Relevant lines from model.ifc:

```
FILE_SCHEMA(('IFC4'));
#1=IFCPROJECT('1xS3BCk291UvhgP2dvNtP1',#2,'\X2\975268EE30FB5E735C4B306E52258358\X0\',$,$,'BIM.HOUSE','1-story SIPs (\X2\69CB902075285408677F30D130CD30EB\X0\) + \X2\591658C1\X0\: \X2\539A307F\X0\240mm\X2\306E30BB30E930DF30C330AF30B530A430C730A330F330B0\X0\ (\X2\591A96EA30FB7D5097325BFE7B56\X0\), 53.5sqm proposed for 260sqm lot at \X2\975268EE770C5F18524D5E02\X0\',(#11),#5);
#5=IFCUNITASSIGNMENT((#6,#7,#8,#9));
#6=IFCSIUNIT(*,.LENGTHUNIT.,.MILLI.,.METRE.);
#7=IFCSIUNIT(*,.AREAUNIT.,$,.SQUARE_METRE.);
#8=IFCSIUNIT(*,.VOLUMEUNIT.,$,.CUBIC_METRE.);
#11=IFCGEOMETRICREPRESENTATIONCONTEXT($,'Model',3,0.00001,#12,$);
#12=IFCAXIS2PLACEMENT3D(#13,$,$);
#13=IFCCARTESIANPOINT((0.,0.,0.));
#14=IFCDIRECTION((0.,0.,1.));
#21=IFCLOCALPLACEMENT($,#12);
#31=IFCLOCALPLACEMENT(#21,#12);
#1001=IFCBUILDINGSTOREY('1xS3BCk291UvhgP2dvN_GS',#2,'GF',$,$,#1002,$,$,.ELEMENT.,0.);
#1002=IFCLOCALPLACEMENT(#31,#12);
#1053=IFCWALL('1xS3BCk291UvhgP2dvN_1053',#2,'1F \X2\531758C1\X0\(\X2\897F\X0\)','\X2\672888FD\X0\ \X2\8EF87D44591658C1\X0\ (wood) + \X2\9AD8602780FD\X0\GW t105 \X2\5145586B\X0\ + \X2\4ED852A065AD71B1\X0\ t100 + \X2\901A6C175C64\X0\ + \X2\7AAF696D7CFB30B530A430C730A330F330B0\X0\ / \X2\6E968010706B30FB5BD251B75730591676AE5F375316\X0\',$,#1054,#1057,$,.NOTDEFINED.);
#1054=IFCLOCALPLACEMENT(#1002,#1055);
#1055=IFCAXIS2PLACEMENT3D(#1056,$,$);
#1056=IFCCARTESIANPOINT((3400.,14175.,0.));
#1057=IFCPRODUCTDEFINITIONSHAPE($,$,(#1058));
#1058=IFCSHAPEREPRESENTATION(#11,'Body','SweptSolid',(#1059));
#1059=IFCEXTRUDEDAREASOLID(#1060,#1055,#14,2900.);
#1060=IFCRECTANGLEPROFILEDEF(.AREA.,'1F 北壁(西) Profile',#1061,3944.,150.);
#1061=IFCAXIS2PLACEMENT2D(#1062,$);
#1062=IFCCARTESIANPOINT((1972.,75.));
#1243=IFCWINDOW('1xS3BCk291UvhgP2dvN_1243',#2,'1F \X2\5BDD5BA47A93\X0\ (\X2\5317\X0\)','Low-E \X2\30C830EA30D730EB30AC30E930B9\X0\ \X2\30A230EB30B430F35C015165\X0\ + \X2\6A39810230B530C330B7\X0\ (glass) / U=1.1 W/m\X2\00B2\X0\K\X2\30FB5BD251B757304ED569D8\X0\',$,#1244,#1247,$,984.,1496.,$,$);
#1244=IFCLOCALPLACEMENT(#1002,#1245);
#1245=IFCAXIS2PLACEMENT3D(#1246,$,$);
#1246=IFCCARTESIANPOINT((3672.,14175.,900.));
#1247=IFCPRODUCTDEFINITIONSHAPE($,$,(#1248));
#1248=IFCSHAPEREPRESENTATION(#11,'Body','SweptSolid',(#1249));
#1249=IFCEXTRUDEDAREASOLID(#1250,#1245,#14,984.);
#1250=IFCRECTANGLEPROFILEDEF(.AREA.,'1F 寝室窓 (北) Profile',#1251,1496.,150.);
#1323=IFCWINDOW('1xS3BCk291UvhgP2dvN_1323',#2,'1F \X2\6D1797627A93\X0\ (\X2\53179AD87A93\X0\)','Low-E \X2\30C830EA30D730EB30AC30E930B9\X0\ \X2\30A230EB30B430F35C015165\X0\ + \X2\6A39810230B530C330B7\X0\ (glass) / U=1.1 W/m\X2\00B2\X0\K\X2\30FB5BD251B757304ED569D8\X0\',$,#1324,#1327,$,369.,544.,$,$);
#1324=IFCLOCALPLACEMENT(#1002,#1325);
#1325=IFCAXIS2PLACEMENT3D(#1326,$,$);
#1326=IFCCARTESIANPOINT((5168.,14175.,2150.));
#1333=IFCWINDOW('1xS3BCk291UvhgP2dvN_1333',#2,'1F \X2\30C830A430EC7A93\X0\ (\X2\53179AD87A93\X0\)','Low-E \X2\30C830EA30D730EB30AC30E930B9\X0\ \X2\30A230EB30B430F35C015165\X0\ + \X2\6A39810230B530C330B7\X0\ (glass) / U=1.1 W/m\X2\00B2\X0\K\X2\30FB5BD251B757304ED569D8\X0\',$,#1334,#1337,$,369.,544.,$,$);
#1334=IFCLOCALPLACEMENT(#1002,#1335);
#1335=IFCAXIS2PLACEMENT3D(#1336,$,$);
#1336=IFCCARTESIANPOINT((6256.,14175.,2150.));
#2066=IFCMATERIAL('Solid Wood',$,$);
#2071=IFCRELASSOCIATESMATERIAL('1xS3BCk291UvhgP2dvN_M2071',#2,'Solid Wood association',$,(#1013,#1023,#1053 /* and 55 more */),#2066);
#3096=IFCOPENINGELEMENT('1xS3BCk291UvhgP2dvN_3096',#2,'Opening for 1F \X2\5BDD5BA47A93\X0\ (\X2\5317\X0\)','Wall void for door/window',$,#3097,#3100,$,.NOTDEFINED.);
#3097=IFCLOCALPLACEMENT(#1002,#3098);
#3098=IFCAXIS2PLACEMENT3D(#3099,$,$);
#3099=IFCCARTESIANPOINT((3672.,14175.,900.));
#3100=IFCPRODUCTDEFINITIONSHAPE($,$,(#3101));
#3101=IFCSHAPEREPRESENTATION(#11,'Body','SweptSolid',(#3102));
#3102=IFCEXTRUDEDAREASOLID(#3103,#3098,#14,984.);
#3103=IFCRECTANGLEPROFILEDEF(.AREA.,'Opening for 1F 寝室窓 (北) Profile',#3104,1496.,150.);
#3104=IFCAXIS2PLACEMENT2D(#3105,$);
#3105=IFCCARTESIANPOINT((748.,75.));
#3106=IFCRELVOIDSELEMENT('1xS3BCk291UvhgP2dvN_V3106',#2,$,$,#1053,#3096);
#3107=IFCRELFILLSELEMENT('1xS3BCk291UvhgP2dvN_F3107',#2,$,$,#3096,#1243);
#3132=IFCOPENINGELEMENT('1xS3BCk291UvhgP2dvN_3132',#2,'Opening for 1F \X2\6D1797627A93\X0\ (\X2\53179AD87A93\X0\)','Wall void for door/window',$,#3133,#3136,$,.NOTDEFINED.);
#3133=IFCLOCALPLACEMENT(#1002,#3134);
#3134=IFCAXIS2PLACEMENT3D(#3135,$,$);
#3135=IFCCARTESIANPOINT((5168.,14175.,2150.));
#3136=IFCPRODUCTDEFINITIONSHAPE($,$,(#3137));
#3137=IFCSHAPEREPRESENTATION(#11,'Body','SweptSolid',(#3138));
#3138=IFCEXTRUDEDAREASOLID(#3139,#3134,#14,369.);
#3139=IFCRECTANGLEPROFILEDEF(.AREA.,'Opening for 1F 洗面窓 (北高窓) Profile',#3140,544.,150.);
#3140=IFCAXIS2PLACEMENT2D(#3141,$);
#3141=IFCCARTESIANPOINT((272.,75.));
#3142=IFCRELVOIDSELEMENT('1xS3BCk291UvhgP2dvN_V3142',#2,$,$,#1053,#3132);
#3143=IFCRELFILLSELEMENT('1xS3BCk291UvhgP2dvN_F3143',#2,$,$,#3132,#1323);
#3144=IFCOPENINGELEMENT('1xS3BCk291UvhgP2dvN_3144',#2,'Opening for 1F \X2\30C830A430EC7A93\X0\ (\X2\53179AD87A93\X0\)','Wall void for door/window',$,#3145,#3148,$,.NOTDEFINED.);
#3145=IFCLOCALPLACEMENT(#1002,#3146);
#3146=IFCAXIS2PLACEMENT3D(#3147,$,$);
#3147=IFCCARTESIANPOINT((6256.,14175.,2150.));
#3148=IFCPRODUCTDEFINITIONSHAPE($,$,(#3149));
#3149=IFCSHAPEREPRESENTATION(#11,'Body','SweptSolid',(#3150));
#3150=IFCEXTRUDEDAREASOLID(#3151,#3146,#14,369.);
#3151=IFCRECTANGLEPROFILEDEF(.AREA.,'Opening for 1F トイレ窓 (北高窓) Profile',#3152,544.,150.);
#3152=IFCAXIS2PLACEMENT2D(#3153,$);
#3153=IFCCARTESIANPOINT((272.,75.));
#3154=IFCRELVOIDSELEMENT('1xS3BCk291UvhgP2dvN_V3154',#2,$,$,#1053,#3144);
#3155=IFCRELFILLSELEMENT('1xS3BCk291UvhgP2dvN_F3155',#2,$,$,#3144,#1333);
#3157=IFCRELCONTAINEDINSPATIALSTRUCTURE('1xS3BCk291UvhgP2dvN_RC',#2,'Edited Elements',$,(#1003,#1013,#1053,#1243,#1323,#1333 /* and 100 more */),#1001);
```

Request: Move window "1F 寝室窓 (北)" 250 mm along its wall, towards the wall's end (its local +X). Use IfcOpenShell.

```python
import ifcopenshell
import ifcopenshell.api.geometry
import ifcopenshell.util.placement
import ifcopenshell.util.unit

model = ifcopenshell.open("model.ifc")
unit_scale = ifcopenshell.util.unit.calculate_unit_scale(model)

window = model.by_guid("1xS3BCk291UvhgP2dvN_1243")
opening = window.FillsVoids[0].RelatingOpeningElement
wall = opening.VoidsElements[0].RelatingBuildingElement

wall_matrix = ifcopenshell.util.placement.get_local_placement(wall.ObjectPlacement)
shift = wall_matrix[:3, 0] * 0.25 / unit_scale
before = ifcopenshell.util.placement.get_local_placement(window.ObjectPlacement)[:3, 3].copy()

# The window is not placed relative to its opening, so move both.
for product in (opening, window):
    matrix = ifcopenshell.util.placement.get_local_placement(product.ObjectPlacement)
    matrix[:3, 3] += shift
    ifcopenshell.api.geometry.edit_object_placement(model, product=product, matrix=matrix, is_si=False)

after = ifcopenshell.util.placement.get_local_placement(window.ObjectPlacement)[:3, 3]
print("window moved by", (after - before).round(3) + 0.0)

model.write("model_v2.ifc")
```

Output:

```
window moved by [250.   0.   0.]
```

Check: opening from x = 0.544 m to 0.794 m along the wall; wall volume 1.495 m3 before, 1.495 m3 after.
